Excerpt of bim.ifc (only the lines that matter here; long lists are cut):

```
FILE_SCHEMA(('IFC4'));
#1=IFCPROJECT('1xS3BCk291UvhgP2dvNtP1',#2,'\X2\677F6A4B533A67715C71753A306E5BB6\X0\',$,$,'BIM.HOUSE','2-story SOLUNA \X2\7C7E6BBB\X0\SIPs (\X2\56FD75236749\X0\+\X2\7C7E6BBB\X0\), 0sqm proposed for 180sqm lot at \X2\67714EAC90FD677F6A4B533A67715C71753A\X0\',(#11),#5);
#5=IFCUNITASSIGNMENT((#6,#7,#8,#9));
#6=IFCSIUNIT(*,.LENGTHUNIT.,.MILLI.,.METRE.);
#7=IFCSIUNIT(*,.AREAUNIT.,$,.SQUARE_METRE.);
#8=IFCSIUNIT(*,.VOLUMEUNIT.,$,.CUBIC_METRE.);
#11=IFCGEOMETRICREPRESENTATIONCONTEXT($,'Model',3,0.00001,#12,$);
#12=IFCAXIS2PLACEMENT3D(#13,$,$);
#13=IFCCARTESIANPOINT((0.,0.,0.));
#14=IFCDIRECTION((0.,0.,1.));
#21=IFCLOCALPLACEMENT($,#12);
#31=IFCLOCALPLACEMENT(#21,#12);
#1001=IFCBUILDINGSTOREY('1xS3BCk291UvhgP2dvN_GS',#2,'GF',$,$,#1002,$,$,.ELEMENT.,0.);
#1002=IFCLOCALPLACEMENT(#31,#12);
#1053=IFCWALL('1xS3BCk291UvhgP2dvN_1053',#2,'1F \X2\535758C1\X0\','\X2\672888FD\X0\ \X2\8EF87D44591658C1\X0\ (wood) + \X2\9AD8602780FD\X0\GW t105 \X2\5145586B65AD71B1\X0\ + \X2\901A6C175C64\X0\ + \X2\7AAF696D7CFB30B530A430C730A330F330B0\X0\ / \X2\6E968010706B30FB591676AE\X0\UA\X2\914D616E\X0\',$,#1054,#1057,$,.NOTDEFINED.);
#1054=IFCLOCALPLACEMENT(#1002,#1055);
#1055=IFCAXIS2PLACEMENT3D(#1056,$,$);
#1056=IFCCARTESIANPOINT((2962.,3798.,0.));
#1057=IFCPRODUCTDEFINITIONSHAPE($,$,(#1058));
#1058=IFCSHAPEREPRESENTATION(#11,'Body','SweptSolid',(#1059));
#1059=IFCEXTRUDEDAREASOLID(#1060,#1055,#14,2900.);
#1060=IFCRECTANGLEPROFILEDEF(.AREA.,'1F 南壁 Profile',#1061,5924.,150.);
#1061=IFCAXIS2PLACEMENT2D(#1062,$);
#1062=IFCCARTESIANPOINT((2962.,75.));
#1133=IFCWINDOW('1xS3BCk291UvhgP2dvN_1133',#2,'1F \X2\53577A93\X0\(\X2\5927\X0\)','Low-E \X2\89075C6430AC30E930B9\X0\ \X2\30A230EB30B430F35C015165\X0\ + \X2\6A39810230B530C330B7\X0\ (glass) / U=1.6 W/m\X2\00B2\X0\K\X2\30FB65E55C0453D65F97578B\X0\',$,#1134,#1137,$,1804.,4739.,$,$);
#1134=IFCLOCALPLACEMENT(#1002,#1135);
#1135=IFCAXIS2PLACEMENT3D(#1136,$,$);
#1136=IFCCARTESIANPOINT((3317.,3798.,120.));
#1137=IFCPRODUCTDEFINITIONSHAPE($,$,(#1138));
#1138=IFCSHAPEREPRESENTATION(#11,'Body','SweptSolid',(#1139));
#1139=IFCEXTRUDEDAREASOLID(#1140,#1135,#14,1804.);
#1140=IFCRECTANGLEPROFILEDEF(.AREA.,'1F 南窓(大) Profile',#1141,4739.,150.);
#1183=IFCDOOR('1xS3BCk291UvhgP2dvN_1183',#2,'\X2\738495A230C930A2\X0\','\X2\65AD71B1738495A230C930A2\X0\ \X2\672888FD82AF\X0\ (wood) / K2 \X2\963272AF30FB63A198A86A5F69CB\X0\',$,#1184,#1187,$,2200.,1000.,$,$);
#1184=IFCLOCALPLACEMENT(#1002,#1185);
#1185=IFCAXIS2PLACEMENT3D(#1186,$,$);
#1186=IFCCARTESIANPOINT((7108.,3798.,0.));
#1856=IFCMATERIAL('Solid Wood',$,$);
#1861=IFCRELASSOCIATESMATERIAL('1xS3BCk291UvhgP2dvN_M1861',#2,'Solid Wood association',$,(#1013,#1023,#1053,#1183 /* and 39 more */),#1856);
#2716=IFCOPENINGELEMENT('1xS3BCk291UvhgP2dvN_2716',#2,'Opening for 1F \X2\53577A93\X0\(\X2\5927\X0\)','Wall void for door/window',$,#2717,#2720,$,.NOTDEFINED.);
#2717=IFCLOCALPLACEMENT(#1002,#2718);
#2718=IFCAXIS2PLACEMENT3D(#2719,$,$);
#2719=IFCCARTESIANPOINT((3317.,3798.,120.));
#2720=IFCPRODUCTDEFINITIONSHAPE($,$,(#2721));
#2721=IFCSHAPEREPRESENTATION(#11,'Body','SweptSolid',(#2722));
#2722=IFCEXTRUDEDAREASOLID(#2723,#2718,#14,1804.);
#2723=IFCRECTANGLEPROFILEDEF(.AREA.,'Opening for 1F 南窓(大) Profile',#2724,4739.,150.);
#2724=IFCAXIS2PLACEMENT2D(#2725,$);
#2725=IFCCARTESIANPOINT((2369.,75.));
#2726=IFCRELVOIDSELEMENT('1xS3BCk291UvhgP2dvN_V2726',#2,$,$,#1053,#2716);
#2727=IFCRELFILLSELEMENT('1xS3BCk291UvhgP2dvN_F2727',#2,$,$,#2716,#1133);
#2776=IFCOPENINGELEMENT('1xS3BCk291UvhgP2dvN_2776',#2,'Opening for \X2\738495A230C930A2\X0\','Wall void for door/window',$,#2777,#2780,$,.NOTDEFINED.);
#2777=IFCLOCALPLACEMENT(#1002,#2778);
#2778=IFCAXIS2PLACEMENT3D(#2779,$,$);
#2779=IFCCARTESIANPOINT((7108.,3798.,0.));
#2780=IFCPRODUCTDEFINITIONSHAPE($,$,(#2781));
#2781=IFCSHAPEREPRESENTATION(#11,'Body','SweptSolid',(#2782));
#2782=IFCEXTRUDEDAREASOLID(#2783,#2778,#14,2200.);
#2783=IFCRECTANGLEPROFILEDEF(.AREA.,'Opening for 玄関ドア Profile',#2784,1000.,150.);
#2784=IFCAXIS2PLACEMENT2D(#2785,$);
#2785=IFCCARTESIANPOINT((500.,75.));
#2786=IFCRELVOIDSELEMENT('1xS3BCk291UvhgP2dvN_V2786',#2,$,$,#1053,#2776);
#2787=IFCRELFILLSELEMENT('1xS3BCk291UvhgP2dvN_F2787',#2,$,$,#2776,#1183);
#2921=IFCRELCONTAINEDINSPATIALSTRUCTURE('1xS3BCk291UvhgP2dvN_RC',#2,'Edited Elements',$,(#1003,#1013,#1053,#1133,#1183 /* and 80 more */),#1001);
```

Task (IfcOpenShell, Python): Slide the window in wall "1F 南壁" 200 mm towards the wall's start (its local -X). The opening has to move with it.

```python
import ifcopenshell
import ifcopenshell.api.geometry
import ifcopenshell.util.placement

model = ifcopenshell.open("bim.ifc")

window = model.by_guid("1xS3BCk291UvhgP2dvN_1133")
opening = window.FillsVoids[0].RelatingOpeningElement
wall = opening.VoidsElements[0].RelatingBuildingElement

wall_matrix = ifcopenshell.util.placement.get_local_placement(wall.ObjectPlacement)
shift = wall_matrix[:3, 0] * -200.0
before = ifcopenshell.util.placement.get_local_placement(window.ObjectPlacement)[:3, 3].copy()

# The window is not placed relative to its opening, so move both.
for product in (opening, window):
    matrix = ifcopenshell.util.placement.get_local_placement(product.ObjectPlacement)
    matrix[:3, 3] += shift
    ifcopenshell.api.geometry.edit_object_placement(model, product=product, matrix=matrix, is_si=False)

after = ifcopenshell.util.placement.get_local_placement(window.ObjectPlacement)[:3, 3]
print("window moved by", (after - before).round(3) + 0.0)

model.write("bim-out.ifc")
```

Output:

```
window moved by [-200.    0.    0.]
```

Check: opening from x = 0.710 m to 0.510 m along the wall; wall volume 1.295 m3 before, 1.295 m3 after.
